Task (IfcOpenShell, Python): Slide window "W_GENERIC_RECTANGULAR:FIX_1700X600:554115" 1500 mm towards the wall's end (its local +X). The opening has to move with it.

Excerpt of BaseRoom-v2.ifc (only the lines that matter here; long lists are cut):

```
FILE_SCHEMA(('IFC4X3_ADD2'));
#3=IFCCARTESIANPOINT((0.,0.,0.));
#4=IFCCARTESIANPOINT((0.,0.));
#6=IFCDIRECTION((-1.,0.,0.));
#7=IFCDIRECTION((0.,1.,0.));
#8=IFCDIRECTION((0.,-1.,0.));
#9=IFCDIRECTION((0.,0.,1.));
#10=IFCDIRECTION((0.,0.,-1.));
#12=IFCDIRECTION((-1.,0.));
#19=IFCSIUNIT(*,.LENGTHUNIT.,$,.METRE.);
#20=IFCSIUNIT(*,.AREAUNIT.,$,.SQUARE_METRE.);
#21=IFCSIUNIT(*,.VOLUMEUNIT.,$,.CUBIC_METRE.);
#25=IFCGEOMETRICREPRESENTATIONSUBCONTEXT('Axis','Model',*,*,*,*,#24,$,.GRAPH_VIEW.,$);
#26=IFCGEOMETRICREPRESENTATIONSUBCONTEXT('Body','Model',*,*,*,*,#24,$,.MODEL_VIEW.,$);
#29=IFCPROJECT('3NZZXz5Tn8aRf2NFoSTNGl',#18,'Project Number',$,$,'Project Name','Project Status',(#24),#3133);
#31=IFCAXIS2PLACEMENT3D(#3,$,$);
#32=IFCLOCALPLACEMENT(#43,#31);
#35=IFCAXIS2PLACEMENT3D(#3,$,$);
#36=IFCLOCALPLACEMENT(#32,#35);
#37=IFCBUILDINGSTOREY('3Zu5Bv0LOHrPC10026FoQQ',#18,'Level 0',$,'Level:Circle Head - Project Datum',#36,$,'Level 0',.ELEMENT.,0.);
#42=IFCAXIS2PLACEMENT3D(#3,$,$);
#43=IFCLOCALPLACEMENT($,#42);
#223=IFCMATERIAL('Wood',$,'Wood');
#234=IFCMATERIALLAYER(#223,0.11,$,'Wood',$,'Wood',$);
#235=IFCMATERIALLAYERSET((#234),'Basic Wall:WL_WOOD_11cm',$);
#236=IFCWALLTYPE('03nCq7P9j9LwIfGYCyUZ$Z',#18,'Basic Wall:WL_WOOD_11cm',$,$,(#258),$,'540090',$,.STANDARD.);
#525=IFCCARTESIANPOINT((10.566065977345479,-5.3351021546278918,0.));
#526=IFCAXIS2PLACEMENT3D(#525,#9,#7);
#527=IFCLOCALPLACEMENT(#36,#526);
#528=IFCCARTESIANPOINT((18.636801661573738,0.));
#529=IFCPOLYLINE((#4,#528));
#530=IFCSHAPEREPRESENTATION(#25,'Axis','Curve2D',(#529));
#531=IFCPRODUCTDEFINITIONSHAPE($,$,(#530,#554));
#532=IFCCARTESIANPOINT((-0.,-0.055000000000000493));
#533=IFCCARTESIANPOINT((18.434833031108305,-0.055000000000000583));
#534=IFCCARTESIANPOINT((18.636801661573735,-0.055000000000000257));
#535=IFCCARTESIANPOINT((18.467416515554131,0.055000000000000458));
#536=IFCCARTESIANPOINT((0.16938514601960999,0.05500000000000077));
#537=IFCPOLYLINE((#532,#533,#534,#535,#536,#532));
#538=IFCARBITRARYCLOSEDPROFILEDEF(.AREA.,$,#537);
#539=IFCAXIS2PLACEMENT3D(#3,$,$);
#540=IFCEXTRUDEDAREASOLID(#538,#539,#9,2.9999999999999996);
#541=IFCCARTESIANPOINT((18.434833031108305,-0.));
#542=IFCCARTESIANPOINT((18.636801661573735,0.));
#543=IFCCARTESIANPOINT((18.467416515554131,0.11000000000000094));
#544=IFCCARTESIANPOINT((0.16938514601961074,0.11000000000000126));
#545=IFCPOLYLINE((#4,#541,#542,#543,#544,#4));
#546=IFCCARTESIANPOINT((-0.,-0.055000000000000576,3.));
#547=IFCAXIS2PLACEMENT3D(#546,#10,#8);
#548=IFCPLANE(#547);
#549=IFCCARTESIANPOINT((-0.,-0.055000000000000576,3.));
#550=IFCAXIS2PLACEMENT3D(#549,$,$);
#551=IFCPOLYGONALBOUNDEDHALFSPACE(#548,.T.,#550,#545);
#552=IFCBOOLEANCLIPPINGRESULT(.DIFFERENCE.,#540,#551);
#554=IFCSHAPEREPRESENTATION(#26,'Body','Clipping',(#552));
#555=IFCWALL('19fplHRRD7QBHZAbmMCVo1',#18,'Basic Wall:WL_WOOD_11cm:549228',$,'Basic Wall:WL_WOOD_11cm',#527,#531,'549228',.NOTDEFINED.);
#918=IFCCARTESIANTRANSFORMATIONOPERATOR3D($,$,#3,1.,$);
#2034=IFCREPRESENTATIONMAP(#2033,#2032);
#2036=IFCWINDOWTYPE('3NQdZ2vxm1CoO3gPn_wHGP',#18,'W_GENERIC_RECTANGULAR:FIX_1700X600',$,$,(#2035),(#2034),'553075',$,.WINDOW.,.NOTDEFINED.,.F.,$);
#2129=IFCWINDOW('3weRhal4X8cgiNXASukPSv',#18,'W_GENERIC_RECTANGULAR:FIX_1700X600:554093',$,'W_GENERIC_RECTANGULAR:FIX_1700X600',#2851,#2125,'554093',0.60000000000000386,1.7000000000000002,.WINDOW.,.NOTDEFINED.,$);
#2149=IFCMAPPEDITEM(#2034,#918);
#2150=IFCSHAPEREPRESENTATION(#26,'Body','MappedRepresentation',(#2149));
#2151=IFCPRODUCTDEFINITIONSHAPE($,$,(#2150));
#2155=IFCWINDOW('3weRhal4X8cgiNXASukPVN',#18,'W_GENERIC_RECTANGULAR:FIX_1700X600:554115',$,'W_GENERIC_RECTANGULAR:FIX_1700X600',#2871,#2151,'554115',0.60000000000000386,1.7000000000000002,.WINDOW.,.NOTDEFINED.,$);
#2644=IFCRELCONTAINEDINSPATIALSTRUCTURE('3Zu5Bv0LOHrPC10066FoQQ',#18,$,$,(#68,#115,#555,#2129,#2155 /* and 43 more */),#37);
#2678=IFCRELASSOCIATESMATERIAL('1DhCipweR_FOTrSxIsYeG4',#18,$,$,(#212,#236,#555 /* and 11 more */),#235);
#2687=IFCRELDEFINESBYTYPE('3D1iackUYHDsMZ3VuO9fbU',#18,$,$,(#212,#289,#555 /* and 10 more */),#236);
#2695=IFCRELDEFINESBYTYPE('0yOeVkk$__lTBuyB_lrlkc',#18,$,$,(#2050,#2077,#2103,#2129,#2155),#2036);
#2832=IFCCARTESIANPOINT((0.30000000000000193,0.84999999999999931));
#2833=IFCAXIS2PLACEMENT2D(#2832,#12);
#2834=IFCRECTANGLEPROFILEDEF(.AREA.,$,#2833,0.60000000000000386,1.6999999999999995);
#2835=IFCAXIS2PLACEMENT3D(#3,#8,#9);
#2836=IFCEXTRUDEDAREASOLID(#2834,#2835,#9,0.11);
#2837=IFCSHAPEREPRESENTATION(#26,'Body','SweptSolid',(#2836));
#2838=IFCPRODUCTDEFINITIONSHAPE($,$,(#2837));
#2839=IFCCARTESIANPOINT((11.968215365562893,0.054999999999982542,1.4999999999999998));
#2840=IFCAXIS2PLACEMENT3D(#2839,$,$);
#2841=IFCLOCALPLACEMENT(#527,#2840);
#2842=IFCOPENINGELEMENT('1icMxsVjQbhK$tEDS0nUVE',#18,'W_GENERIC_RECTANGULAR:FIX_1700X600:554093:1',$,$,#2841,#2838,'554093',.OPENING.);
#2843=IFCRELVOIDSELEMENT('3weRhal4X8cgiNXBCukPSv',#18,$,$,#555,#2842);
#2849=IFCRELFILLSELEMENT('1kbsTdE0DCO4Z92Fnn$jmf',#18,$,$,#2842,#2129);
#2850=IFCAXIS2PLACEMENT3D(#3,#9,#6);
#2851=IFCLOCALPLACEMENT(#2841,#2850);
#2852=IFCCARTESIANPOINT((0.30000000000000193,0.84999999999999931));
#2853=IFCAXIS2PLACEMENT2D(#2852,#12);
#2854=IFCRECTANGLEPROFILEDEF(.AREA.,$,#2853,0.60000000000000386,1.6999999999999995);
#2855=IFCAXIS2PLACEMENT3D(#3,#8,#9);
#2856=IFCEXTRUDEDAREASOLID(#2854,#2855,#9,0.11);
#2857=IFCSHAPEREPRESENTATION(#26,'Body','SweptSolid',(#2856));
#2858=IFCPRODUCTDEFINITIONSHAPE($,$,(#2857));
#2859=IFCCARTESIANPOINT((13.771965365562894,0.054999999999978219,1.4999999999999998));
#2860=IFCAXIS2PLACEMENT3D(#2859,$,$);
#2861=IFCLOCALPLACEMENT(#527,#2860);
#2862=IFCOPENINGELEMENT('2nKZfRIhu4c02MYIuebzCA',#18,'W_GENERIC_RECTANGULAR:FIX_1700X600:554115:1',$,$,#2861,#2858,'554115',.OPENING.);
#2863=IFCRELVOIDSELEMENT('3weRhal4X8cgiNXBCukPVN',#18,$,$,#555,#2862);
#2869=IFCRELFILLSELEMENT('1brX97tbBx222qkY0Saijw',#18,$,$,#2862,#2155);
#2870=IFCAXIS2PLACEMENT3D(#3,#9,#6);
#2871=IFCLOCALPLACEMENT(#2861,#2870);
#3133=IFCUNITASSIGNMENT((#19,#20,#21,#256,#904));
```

```python
import ifcopenshell
import ifcopenshell.api.geometry
import ifcopenshell.util.placement
import ifcopenshell.util.unit

model = ifcopenshell.open("BaseRoom-v2.ifc")
unit_scale = ifcopenshell.util.unit.calculate_unit_scale(model)

window = model.by_guid("3weRhal4X8cgiNXASukPVN")
opening = window.FillsVoids[0].RelatingOpeningElement
wall = opening.VoidsElements[0].RelatingBuildingElement

wall_matrix = ifcopenshell.util.placement.get_local_placement(wall.ObjectPlacement)
shift = wall_matrix[:3, 0] * 1.5 / unit_scale
before = ifcopenshell.util.placement.get_local_placement(window.ObjectPlacement)[:3, 3].copy()

# The window is placed relative to its opening, so it follows when the opening moves.
matrix = ifcopenshell.util.placement.get_local_placement(opening.ObjectPlacement)
matrix[:3, 3] += shift
ifcopenshell.api.geometry.edit_object_placement(
    model, product=opening, matrix=matrix, is_si=False, should_transform_children=True
)

after = ifcopenshell.util.placement.get_local_placement(window.ObjectPlacement)[:3, 3]
print("window moved by", (after - before).round(3) + 0.0)

model.write("BaseRoom-v2-out.ifc")
```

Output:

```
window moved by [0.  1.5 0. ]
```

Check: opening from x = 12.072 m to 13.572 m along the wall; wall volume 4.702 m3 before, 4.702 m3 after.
